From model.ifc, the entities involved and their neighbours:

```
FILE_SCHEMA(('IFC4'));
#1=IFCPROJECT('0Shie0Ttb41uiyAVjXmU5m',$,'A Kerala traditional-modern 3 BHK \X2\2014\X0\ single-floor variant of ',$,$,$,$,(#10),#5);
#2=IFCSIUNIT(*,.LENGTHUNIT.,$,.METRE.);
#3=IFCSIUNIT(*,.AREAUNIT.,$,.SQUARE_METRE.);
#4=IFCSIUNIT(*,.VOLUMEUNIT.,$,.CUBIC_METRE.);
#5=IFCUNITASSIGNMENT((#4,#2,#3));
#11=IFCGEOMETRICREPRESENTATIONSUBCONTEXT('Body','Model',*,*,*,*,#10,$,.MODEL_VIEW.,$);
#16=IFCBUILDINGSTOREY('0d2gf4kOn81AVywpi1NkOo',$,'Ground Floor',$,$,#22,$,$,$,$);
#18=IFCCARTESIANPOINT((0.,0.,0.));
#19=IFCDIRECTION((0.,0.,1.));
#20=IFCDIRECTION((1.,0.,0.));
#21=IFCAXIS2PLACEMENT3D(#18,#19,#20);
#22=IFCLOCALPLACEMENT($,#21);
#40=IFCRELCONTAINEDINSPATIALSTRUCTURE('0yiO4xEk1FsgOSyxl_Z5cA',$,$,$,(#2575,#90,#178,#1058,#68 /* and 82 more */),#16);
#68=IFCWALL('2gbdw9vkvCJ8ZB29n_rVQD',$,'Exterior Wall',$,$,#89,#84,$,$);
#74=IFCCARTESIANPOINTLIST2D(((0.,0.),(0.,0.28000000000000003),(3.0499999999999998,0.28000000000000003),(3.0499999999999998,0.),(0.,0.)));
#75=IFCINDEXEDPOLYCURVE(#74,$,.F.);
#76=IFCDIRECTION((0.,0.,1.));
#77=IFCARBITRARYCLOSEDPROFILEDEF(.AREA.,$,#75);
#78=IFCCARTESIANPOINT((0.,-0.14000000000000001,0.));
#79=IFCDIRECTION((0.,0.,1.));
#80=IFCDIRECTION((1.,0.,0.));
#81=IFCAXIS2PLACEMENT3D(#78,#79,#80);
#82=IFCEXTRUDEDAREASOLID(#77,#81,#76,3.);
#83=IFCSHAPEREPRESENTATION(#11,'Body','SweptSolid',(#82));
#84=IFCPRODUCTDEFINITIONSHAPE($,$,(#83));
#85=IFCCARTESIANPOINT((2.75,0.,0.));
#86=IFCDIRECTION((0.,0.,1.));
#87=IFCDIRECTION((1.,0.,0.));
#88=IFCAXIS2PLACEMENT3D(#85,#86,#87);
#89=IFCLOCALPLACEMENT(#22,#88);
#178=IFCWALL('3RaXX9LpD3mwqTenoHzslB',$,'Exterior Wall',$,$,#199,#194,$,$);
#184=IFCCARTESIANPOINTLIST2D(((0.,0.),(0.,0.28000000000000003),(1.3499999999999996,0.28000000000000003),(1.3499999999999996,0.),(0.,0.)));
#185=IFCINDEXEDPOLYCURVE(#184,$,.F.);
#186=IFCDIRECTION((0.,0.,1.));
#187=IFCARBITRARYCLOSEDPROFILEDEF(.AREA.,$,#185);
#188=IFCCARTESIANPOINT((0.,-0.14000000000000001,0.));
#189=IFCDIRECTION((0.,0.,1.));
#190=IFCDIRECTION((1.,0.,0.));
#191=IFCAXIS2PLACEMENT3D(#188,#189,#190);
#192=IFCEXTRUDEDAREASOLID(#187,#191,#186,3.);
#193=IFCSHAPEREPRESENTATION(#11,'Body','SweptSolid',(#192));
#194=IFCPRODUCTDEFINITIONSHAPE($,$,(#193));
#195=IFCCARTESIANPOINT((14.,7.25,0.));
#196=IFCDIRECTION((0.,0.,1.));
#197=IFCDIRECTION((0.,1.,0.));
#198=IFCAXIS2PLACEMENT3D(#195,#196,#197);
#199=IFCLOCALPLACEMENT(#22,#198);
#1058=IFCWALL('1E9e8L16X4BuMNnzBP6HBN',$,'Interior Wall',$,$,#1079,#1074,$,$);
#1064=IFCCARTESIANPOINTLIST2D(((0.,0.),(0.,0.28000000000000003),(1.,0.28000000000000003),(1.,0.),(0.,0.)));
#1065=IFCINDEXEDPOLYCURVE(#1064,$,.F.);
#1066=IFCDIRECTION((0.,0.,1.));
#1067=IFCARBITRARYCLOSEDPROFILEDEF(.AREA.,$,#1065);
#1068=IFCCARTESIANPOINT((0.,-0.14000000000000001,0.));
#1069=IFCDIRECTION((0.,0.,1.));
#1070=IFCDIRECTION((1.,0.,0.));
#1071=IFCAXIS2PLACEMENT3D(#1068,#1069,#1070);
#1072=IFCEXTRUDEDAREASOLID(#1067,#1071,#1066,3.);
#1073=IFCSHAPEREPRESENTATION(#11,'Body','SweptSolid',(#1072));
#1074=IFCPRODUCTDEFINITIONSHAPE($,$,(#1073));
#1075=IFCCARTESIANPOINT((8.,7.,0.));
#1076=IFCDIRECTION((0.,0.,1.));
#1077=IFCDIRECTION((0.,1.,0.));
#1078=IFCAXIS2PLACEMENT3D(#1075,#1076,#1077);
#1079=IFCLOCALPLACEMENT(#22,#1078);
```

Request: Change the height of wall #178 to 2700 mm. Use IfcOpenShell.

```python
import ifcopenshell
import ifcopenshell.geom
import ifcopenshell.util.representation
import ifcopenshell.util.shape

model = ifcopenshell.open("model.ifc")
settings = ifcopenshell.geom.settings()


def volume(element):
    """Net volume in cubic metres, openings subtracted."""
    shape = ifcopenshell.geom.create_shape(settings, element)
    return ifcopenshell.util.shape.get_volume(shape.geometry)


wall = model.by_guid("3RaXX9LpD3mwqTenoHzslB")
before = volume(wall)

body = ifcopenshell.util.representation.get_representation(wall, "Model", "Body")
solid = body.Items[0]
old_height = solid.Depth
solid.Depth = 2.7
after = volume(wall)

print(f"height {old_height:g} -> {solid.Depth:g}, volume {before:.3f} -> {after:.3f} m3")

model.write("model_edited.ifc")
```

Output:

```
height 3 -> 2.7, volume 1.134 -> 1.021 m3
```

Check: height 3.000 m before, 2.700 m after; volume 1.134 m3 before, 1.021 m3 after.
